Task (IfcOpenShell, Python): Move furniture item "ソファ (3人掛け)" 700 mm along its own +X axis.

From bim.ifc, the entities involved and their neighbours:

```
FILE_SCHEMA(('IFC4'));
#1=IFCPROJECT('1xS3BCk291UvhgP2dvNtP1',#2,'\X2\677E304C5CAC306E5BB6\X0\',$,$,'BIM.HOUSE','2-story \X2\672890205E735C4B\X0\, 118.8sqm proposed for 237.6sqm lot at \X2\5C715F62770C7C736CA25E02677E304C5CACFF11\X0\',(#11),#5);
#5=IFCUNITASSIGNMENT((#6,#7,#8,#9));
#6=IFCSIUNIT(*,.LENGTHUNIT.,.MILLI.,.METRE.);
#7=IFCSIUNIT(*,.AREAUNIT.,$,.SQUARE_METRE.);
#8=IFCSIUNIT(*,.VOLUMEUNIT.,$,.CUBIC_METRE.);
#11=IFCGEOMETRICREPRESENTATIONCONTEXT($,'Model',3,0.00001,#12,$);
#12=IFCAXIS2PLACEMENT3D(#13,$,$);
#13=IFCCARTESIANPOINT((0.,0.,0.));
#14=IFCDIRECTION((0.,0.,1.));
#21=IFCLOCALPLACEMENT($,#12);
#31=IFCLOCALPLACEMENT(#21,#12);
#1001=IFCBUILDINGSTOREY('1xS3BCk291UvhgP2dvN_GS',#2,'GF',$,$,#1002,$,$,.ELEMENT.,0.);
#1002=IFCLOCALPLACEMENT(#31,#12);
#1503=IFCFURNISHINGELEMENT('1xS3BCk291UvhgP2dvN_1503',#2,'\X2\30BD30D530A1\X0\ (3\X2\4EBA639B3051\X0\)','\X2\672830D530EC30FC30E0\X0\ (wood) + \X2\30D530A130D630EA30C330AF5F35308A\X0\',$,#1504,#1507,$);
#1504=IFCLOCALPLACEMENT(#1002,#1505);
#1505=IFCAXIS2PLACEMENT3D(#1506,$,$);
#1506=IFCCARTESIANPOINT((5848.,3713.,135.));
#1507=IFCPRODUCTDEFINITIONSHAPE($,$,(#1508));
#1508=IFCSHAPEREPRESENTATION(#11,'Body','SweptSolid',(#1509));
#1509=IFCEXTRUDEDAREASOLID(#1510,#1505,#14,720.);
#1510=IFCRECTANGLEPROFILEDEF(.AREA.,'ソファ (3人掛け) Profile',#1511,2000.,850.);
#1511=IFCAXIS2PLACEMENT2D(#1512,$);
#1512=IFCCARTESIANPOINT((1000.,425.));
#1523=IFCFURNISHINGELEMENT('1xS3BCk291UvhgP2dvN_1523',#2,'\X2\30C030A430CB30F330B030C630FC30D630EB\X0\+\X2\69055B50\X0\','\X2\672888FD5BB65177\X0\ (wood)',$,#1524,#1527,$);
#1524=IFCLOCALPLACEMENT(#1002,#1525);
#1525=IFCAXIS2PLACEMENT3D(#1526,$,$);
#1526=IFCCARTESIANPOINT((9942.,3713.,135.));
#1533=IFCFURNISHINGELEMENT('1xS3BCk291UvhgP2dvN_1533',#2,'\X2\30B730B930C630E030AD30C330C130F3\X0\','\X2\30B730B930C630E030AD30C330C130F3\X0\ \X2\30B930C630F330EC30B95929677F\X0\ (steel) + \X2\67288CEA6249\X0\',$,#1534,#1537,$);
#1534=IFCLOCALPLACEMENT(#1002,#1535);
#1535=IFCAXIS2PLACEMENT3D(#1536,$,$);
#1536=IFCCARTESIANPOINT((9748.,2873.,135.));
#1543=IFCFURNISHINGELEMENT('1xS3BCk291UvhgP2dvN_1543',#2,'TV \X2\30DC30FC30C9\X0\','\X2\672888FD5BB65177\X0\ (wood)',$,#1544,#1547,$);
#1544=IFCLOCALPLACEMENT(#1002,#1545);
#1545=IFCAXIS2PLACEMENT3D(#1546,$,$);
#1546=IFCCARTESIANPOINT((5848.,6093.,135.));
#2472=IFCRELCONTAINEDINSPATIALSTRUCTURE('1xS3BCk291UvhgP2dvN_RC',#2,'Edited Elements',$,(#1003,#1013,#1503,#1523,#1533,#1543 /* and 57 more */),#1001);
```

```python
import ifcopenshell
import ifcopenshell.api.geometry
import ifcopenshell.util.placement
import ifcopenshell.util.unit

model = ifcopenshell.open("bim.ifc")
unit_scale = ifcopenshell.util.unit.calculate_unit_scale(model)

item = model.by_id(1503)
matrix = ifcopenshell.util.placement.get_local_placement(item.ObjectPlacement)
matrix[:3, 3] += matrix[:3, 0] * 0.7 / unit_scale
ifcopenshell.api.geometry.edit_object_placement(model, product=item, matrix=matrix, is_si=False)

print(ifcopenshell.util.placement.get_local_placement(item.ObjectPlacement).round(3) + 0.0)

model.write("bim_rev.ifc")
```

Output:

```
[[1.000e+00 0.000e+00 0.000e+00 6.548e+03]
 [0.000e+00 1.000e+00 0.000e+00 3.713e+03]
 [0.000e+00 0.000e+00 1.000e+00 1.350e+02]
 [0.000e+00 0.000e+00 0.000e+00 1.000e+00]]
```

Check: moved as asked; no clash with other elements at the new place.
